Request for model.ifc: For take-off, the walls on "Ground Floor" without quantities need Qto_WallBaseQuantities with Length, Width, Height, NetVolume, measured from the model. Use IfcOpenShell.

First a look at what the model holds.

```python
import ifcopenshell
import ifcopenshell.util.element
import ifcopenshell.util.unit

model = ifcopenshell.open("model.ifc")
print(model.schema)
for unit_type in ("LENGTHUNIT", "AREAUNIT", "VOLUMEUNIT"):
    print(unit_type, ifcopenshell.util.unit.calculate_unit_scale(model, unit_type))
storey = next(s for s in model.by_type("IfcBuildingStorey") if s.Name == "Ground Floor")
walls = [e for e in ifcopenshell.util.element.get_decomposition(storey) if e.is_a("IfcWall")]
for e in sorted(walls, key=lambda e: e.id()):
    print(e.id(), e.is_a(), e.Name, list(ifcopenshell.util.element.get_psets(e, qtos_only=True)), sep=" | ")
```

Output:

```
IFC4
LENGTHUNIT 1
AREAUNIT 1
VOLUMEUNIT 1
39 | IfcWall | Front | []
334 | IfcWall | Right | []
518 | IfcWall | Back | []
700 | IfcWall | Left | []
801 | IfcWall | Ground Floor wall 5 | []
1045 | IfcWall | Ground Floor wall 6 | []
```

```python
import ifcopenshell
import ifcopenshell.api.pset
import ifcopenshell.geom
import ifcopenshell.util.element
import ifcopenshell.util.shape
import ifcopenshell.util.unit

model = ifcopenshell.open("model.ifc")
unit_scale = ifcopenshell.util.unit.calculate_unit_scale(model)
volume_scale = ifcopenshell.util.unit.calculate_unit_scale(model, "VOLUMEUNIT")
settings = ifcopenshell.geom.settings()

storey = next(s for s in model.by_type("IfcBuildingStorey") if s.Name == "Ground Floor")
walls = [e for e in ifcopenshell.util.element.get_decomposition(storey) if e.is_a("IfcWall")]

for e in sorted(walls, key=lambda e: e.id()):
    if ifcopenshell.util.element.get_psets(e, qtos_only=True, should_inherit=False):
        continue
    # Geometry comes back in metres, in the element's own axes.
    shape = ifcopenshell.geom.create_shape(settings, e)
    values = {
        "Length": ifcopenshell.util.shape.get_x(shape.geometry) / unit_scale,
        "Width": ifcopenshell.util.shape.get_y(shape.geometry) / unit_scale,
        "Height": ifcopenshell.util.shape.get_z(shape.geometry) / unit_scale,
        "NetVolume": ifcopenshell.util.shape.get_volume(shape.geometry) / volume_scale,
    }
    qto = ifcopenshell.api.pset.add_qto(model, product=e, name="Qto_WallBaseQuantities")
    ifcopenshell.api.pset.edit_qto(model, qto=qto, properties=values)
    print(e.id(), {k: round(v, 3) for k, v in values.items()})

model.write("model_v2.ifc")
```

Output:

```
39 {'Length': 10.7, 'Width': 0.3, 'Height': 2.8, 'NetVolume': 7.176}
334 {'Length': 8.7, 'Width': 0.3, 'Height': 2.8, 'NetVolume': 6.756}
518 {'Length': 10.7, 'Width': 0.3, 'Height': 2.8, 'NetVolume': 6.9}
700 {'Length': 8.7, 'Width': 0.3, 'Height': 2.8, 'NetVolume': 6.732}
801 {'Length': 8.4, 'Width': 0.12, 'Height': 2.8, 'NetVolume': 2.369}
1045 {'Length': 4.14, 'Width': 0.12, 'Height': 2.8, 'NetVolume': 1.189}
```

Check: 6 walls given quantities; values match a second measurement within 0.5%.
